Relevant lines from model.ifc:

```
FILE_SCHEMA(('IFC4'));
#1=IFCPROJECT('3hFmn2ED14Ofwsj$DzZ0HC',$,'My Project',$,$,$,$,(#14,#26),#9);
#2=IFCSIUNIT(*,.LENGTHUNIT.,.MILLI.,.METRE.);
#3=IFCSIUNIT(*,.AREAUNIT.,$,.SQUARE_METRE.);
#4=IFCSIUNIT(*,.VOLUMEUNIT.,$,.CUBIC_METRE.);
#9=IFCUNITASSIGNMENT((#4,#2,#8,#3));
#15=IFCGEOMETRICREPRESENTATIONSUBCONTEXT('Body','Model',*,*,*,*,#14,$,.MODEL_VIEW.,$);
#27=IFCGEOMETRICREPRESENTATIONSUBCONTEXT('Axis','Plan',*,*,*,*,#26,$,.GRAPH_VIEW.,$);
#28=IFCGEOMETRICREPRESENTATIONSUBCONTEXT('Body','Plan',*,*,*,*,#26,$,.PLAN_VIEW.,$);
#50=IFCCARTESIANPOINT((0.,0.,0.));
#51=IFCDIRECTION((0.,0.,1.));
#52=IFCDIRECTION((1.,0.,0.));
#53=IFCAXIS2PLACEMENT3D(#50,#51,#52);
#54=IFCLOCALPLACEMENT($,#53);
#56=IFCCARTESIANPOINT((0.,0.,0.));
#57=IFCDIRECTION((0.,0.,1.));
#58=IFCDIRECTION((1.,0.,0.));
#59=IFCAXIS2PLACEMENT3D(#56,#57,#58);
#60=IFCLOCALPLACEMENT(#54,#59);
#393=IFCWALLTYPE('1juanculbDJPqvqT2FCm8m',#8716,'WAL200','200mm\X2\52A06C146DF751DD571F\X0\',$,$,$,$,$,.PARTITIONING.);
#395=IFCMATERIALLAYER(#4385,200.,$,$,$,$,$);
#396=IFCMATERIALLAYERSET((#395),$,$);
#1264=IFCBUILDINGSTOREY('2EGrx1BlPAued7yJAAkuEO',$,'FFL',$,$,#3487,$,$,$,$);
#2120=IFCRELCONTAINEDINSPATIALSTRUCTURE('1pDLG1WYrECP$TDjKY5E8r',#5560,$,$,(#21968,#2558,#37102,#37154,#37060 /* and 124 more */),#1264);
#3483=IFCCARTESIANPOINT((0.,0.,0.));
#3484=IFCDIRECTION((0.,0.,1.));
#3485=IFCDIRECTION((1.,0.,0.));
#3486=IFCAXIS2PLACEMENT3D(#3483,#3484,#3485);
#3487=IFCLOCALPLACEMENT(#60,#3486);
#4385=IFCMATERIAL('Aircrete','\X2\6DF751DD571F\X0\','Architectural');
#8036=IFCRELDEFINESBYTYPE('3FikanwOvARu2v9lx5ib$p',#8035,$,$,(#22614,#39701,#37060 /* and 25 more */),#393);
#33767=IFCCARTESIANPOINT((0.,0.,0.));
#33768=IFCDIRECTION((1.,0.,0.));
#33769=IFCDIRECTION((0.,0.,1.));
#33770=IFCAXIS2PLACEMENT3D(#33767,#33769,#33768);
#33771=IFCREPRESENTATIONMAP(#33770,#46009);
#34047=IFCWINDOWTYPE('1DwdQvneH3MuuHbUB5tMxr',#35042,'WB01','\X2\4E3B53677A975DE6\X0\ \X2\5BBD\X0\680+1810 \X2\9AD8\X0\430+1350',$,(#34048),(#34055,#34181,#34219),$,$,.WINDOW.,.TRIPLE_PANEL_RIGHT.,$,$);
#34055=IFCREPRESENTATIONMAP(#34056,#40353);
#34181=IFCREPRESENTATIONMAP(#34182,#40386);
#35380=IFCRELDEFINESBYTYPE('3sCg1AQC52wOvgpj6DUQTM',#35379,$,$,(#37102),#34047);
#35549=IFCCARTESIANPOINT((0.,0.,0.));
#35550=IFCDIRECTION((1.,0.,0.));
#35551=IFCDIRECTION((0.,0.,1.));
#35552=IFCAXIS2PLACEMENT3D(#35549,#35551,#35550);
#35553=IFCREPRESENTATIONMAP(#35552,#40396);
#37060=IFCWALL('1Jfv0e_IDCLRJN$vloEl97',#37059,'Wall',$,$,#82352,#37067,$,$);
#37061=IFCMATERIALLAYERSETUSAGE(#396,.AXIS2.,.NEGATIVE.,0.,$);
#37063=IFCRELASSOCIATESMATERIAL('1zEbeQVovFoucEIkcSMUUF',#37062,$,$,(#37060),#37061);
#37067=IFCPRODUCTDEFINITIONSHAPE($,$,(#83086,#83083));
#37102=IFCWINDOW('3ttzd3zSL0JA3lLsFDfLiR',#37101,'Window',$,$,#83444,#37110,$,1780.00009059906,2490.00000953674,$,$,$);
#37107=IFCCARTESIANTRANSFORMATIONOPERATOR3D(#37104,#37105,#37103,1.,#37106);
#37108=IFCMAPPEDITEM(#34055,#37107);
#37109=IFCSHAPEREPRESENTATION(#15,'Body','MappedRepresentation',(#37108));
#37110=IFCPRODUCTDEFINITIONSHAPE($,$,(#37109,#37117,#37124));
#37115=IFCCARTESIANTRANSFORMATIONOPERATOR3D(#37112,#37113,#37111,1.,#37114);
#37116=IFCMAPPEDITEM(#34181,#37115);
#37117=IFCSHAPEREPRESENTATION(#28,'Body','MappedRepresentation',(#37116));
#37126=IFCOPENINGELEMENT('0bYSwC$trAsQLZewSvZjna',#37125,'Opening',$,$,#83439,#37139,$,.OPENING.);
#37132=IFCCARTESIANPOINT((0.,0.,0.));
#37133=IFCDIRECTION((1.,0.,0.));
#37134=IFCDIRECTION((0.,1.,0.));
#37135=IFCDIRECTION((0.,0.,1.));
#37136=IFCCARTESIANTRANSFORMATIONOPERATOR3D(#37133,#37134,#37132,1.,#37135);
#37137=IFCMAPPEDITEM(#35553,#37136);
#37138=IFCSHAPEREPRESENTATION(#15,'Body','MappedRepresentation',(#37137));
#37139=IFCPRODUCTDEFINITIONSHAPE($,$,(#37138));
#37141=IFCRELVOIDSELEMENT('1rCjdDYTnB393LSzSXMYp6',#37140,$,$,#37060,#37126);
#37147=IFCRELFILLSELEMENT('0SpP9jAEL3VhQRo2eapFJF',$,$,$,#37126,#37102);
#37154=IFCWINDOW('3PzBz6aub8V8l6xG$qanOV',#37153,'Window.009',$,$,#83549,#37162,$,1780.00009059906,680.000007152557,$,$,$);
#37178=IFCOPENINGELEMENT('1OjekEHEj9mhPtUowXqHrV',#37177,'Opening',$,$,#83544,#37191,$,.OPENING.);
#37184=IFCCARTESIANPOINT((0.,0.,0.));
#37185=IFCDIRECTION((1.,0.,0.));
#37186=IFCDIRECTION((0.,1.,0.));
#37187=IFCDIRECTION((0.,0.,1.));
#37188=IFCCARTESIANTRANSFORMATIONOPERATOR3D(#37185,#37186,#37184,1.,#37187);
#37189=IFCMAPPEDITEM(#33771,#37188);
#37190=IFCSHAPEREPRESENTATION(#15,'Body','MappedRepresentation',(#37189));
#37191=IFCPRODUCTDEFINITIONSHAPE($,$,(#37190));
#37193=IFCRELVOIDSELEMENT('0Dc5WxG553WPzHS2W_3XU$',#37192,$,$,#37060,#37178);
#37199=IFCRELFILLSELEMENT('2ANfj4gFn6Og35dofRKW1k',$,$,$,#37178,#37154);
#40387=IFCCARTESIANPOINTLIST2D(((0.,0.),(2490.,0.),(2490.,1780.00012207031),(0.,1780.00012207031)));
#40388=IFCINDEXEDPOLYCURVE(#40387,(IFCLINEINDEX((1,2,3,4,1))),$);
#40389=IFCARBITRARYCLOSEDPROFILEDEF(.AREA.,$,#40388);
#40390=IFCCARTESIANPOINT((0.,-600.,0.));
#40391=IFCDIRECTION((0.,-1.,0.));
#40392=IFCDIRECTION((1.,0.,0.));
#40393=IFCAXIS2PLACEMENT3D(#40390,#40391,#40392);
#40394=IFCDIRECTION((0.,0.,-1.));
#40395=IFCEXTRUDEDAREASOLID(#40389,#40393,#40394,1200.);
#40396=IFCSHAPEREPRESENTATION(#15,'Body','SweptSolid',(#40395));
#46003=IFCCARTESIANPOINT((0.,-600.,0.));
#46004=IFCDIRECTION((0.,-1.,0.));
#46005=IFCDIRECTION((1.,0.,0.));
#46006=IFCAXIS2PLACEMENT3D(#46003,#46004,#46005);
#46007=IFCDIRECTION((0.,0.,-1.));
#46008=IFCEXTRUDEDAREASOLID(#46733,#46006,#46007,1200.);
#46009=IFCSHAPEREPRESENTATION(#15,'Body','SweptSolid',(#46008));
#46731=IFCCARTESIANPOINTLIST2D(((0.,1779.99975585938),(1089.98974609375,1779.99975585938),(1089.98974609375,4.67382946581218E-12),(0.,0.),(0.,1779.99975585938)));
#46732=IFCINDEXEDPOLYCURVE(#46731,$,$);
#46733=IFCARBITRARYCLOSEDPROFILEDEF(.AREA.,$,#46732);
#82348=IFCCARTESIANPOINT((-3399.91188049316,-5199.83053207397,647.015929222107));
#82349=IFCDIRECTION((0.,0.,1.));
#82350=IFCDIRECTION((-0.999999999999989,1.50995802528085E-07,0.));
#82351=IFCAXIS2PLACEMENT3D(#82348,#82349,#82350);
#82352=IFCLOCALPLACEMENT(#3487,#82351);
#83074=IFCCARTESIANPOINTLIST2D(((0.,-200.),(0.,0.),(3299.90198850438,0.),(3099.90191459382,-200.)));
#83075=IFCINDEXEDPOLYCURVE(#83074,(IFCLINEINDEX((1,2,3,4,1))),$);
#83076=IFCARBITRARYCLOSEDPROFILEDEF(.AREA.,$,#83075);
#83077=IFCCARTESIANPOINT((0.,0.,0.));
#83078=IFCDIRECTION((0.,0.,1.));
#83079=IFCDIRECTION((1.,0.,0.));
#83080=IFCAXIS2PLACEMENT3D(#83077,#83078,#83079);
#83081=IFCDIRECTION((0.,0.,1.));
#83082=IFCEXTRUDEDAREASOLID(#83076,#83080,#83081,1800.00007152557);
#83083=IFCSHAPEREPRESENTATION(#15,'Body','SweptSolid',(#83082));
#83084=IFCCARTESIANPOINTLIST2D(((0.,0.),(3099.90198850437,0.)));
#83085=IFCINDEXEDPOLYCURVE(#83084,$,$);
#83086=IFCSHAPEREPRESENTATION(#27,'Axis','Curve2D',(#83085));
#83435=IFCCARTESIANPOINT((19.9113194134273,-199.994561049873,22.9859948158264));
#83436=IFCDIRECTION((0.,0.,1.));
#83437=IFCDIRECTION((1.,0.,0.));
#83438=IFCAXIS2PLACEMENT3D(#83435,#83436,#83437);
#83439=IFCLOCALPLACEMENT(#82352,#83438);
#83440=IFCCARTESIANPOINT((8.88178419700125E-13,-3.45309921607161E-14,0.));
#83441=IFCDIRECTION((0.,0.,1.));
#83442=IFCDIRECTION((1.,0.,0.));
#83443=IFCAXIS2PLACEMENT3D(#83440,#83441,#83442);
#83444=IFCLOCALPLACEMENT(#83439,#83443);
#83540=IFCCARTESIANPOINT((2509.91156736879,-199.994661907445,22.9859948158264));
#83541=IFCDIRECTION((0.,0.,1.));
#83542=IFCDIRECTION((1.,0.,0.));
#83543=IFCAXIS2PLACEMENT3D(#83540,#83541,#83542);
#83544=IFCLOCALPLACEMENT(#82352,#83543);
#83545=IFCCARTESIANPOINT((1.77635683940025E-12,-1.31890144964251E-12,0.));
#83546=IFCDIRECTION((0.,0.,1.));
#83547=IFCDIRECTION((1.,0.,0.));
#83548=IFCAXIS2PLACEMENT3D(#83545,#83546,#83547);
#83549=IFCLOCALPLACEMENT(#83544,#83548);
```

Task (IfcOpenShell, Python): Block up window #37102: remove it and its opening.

```python
import ifcopenshell
import ifcopenshell.api.feature
import ifcopenshell.api.root
import ifcopenshell.geom
import ifcopenshell.util.shape

model = ifcopenshell.open("model.ifc")
settings = ifcopenshell.geom.settings()


def volume(element):
    """Net volume in cubic metres, openings subtracted."""
    shape = ifcopenshell.geom.create_shape(settings, element)
    return ifcopenshell.util.shape.get_volume(shape.geometry)


window = model.by_id(37102)
opening = window.FillsVoids[0].RelatingOpeningElement
wall = opening.VoidsElements[0].RelatingBuildingElement
before = volume(wall)

ifcopenshell.api.root.remove_product(model, product=window)
ifcopenshell.api.feature.remove_feature(model, feature=opening)

after = volume(wall)

print(f"wall volume {before:.3f} -> {after:.3f} m3")

model.write("model-out.ifc")
```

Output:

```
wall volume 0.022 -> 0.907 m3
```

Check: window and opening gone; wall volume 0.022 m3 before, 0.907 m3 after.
